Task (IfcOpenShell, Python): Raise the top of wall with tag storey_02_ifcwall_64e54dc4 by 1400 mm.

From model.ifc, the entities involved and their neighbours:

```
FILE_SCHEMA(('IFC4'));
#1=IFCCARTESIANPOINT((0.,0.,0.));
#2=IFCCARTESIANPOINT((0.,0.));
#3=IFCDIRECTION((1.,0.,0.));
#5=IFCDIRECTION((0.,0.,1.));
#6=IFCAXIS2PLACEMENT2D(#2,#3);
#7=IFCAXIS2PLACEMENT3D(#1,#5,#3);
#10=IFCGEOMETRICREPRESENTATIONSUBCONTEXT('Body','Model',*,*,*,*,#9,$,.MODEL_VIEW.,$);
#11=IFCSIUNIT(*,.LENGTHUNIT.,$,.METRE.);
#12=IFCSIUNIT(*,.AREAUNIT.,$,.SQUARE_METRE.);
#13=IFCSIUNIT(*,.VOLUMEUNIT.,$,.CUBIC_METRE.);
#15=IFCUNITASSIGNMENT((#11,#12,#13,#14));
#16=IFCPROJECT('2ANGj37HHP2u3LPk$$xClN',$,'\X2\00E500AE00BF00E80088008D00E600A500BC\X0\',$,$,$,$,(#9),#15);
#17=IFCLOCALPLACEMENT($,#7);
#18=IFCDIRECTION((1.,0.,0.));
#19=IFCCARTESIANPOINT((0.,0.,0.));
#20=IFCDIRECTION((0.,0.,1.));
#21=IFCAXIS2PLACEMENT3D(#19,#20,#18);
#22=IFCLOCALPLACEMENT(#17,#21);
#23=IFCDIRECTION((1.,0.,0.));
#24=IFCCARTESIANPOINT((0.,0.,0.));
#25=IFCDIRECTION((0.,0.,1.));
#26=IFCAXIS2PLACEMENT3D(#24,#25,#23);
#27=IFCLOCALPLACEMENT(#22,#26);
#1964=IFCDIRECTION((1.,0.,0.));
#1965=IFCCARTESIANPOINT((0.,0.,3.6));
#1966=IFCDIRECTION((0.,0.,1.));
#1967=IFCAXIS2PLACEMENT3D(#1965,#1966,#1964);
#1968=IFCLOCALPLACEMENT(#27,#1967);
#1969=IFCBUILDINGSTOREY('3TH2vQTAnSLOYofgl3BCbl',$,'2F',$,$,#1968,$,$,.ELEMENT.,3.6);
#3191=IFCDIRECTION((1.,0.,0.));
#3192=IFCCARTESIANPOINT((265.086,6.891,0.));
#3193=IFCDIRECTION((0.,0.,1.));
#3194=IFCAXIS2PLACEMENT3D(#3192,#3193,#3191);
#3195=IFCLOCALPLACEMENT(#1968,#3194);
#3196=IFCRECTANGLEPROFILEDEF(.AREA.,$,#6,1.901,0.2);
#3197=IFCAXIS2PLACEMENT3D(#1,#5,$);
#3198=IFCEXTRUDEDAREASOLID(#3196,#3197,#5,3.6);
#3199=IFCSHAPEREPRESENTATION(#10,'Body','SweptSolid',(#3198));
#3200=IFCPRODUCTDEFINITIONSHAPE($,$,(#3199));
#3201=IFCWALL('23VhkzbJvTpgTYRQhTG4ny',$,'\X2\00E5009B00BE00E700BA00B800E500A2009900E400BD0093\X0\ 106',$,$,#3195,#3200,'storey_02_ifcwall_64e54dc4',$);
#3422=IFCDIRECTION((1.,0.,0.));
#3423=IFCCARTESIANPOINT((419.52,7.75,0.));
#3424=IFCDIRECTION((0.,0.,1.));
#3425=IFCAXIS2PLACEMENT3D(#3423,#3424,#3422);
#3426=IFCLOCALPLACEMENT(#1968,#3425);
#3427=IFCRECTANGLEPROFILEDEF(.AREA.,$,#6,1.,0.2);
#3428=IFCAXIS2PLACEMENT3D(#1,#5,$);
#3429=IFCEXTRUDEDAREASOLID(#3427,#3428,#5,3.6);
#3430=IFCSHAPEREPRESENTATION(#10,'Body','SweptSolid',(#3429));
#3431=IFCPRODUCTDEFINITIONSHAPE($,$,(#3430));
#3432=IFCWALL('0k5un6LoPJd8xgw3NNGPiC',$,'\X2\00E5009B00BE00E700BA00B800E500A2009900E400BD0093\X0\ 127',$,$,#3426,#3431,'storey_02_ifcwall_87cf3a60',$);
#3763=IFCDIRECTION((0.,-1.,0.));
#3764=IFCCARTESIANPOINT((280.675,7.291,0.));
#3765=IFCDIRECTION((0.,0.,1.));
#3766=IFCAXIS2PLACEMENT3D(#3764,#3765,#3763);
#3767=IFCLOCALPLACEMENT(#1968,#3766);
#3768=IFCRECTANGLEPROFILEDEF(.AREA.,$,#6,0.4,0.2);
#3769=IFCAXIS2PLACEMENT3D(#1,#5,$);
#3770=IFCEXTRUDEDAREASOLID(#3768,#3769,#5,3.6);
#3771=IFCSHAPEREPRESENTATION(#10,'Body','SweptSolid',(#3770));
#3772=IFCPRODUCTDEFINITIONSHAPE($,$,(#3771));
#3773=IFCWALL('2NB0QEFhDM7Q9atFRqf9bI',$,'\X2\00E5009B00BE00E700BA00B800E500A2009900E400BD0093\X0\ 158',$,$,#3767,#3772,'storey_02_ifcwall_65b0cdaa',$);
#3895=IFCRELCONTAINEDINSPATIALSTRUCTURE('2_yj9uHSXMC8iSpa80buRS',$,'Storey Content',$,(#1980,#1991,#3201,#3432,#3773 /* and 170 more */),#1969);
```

```python
import ifcopenshell
import ifcopenshell.geom
import ifcopenshell.util.representation
import ifcopenshell.util.shape

model = ifcopenshell.open("model.ifc")
settings = ifcopenshell.geom.settings()


def volume(element):
    """Net volume in cubic metres, openings subtracted."""
    shape = ifcopenshell.geom.create_shape(settings, element)
    return ifcopenshell.util.shape.get_volume(shape.geometry)


wall = model.by_id(3201)
before = volume(wall)

body = ifcopenshell.util.representation.get_representation(wall, "Model", "Body")
solid = body.Items[0]
old_height = solid.Depth
solid.Depth += 1.4
after = volume(wall)

print(f"height {old_height:g} -> {solid.Depth:g}, volume {before:.3f} -> {after:.3f} m3")

model.write("model_v2.ifc")
```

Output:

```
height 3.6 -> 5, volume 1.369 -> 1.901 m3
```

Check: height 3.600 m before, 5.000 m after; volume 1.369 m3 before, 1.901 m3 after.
